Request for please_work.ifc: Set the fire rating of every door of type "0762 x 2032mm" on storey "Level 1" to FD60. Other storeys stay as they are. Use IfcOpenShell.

First a look at what the model holds.

```python
import ifcopenshell
import ifcopenshell.util.element

model = ifcopenshell.open("please_work.ifc")
print(model.schema)
storey = next(s for s in model.by_type("IfcBuildingStorey") if s.Name == "Level 1")
doors = [e for e in ifcopenshell.util.element.get_decomposition(storey) if e.is_a("IfcDoor")]
seen = {}
for e in doors:
    element_type = ifcopenshell.util.element.get_type(e)
    key = (element_type.Name if element_type != e and element_type else None, ifcopenshell.util.element.get_pset(e, "Pset_DoorCommon", "FireRating"))
    seen[key] = seen.get(key, 0) + 1
for (name, value), count in sorted(seen.items(), key=str):
    print(count, "x", name, "|", value)
```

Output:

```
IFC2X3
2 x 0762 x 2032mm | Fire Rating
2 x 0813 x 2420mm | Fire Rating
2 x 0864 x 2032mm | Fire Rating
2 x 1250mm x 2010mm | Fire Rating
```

```python
import ifcopenshell
import ifcopenshell.api.pset
import ifcopenshell.util.element

model = ifcopenshell.open("please_work.ifc")

storey = next(s for s in model.by_type("IfcBuildingStorey") if s.Name == "Level 1")
doors = [e for e in ifcopenshell.util.element.get_decomposition(storey) if e.is_a("IfcDoor")]

count = 0
for e in doors:
    element_type = ifcopenshell.util.element.get_type(e)
    if element_type in (None, e) or element_type.Name != "0762 x 2032mm":
        continue
    # add_pset returns the element's existing set when there is one.
    pset = ifcopenshell.api.pset.add_pset(model, product=e, name="Pset_DoorCommon")
    ifcopenshell.api.pset.edit_pset(model, pset=pset, properties={"FireRating": "FD60"})
    count += 1

print(count, "doors updated")

model.write("please_work-out.ifc")
```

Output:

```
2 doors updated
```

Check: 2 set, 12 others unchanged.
